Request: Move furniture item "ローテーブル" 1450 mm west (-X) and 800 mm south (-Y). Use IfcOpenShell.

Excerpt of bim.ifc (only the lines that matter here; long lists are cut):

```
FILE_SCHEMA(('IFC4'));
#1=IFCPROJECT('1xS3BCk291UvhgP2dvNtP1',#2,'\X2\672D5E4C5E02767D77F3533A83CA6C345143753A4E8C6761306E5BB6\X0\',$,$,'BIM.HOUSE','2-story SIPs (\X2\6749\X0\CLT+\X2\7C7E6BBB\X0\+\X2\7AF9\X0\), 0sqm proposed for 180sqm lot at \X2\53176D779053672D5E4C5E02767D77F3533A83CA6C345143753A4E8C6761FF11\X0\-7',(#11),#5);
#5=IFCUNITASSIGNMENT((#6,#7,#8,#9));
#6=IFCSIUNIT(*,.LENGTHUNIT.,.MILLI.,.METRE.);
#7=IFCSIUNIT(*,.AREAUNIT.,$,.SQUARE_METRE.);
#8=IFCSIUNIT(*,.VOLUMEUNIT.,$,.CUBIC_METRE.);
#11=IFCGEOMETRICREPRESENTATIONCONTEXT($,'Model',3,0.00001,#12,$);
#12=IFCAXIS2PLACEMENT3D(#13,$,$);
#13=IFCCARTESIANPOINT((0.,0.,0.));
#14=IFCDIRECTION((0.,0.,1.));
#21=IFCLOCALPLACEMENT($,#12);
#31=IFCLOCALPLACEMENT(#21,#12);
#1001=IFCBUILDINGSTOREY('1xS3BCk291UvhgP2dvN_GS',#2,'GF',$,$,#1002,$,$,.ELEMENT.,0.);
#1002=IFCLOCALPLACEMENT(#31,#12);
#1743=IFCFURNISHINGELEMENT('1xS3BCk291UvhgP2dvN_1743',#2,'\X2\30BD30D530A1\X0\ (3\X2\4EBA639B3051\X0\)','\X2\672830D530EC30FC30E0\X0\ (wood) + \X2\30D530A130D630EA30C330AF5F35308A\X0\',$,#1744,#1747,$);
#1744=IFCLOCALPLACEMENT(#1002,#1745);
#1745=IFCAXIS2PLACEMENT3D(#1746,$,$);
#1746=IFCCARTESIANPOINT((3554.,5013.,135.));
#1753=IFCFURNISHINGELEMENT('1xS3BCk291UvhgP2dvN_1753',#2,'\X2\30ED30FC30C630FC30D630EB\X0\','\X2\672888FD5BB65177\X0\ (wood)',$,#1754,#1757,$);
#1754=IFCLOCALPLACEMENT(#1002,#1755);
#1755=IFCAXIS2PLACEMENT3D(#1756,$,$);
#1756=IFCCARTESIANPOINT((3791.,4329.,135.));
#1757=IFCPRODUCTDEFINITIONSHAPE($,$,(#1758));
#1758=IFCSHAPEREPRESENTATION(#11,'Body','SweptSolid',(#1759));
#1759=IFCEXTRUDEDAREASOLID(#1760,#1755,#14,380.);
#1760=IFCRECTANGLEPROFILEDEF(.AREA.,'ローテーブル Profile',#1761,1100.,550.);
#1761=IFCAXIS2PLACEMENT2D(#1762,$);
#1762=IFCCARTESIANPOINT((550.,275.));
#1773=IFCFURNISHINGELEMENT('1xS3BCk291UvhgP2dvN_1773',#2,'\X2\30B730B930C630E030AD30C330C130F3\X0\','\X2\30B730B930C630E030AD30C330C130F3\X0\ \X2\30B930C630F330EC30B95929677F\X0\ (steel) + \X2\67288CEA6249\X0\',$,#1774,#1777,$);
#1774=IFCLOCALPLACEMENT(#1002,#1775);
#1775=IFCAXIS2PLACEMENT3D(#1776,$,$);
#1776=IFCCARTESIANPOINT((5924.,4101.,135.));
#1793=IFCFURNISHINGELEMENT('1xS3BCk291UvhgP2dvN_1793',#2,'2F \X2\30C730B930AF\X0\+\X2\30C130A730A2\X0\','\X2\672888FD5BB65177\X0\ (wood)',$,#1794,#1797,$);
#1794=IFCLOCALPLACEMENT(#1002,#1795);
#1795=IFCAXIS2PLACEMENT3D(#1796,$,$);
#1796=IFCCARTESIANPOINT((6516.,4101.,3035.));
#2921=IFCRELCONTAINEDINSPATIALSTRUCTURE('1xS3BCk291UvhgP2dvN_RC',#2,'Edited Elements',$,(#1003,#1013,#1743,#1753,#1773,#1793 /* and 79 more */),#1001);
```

```python
import ifcopenshell
import ifcopenshell.api.geometry
import ifcopenshell.util.placement
import ifcopenshell.util.unit

model = ifcopenshell.open("bim.ifc")
unit_scale = ifcopenshell.util.unit.calculate_unit_scale(model)

item = model.by_guid("1xS3BCk291UvhgP2dvN_1753")
matrix = ifcopenshell.util.placement.get_local_placement(item.ObjectPlacement)
matrix[0, 3] -= 1.45 / unit_scale
matrix[1, 3] -= 0.8 / unit_scale
ifcopenshell.api.geometry.edit_object_placement(model, product=item, matrix=matrix, is_si=False)

print(ifcopenshell.util.placement.get_local_placement(item.ObjectPlacement).round(3) + 0.0)

model.write("bim_edited.ifc")
```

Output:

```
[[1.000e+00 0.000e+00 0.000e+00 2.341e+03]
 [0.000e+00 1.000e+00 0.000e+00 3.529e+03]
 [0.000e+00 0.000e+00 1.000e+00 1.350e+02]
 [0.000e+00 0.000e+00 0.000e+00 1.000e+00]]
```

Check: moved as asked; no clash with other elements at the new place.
